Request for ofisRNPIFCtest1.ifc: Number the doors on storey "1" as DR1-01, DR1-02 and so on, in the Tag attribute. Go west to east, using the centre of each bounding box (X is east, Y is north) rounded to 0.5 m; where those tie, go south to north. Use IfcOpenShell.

First a look at what the model holds.

```python
import ifcopenshell
import ifcopenshell.util.element
import ifcopenshell.util.placement

model = ifcopenshell.open("ofisRNPIFCtest1.ifc")
print(model.schema)
storey = next(s for s in model.by_type("IfcBuildingStorey") if s.Name == "1")
doors = [e for e in ifcopenshell.util.element.get_decomposition(storey) if e.is_a("IfcDoor")]
for e in sorted(doors, key=lambda e: e.id()):
    origin = ifcopenshell.util.placement.get_local_placement(e.ObjectPlacement)[:3, 3]
    print(e.id(), e.Tag, e.Name, origin.round(2) + 0.0, sep=" | ")
```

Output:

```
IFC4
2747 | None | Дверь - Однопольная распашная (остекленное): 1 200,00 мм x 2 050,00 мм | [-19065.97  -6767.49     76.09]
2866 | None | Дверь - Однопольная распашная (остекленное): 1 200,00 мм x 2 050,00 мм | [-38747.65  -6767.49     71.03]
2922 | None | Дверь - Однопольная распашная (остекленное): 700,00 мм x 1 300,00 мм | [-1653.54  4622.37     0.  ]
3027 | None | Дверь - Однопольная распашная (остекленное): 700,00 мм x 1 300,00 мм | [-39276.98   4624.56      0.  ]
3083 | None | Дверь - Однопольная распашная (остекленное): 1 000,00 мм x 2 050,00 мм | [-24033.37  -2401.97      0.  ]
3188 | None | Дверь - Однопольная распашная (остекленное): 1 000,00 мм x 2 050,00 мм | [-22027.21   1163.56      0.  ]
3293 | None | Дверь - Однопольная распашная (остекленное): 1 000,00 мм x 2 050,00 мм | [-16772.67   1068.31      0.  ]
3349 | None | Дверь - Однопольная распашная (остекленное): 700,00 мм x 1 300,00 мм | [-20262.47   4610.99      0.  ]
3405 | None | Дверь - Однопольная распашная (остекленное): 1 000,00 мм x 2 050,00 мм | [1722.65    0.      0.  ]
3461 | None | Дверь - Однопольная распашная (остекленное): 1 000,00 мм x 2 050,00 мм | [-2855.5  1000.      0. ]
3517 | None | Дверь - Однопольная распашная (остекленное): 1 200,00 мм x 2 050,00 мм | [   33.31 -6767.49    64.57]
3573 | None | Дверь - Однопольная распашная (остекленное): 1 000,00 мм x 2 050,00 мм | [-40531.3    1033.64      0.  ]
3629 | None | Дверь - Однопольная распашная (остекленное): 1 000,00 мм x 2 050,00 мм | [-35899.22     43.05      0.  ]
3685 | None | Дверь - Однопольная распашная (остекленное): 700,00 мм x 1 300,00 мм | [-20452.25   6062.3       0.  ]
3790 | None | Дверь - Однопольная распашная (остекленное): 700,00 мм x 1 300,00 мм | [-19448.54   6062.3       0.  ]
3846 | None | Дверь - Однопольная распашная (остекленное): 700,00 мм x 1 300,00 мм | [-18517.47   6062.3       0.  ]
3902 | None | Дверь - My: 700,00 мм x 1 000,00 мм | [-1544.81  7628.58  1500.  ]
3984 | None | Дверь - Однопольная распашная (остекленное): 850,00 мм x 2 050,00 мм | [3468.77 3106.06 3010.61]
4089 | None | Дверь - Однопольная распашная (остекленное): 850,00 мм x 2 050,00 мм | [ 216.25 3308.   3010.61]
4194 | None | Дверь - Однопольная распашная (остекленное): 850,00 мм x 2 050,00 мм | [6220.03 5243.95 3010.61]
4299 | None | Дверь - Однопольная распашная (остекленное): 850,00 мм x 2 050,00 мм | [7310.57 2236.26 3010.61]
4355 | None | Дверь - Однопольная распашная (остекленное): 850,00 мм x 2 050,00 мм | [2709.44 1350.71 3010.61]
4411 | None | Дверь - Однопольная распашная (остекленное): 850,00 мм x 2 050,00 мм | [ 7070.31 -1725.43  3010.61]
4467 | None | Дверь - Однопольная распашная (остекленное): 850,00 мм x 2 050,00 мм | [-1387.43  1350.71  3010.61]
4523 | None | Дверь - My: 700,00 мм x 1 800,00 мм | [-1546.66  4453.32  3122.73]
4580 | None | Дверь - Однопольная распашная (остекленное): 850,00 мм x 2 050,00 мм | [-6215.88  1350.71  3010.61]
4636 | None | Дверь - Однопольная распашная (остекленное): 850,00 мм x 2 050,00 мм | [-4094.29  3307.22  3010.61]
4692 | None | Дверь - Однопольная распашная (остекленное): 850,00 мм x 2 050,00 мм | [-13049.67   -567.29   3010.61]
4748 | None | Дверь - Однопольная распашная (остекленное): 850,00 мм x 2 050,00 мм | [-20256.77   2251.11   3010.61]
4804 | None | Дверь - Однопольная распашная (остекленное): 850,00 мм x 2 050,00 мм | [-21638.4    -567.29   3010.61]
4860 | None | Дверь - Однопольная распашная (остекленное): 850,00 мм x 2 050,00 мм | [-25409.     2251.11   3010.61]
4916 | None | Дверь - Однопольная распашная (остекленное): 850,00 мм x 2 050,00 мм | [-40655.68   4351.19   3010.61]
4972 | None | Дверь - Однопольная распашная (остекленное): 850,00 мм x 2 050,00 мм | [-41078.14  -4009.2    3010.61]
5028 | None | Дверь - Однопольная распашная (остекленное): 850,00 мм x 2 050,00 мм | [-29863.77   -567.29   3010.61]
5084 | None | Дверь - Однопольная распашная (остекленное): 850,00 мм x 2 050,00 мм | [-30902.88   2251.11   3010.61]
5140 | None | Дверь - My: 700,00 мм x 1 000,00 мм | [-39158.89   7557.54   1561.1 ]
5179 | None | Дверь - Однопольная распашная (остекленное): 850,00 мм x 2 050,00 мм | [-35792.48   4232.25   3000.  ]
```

```python
import ifcopenshell
import ifcopenshell.geom
import ifcopenshell.util.element
import ifcopenshell.util.shape

model = ifcopenshell.open("ofisRNPIFCtest1.ifc")
settings = ifcopenshell.geom.settings()
settings.set("use-world-coords", True)


def centre(element):
    shape = ifcopenshell.geom.create_shape(settings, element)
    return ifcopenshell.util.shape.get_bbox_centroid(shape.geometry)


storey = next(s for s in model.by_type("IfcBuildingStorey") if s.Name == "1")
doors = [e for e in ifcopenshell.util.element.get_decomposition(storey) if e.is_a("IfcDoor")]

# Insertion points can sit at a corner or the storey origin, so sort by the geometry (in metres).
centres = {e: centre(e) for e in doors}
doors.sort(key=lambda e: (round(centres[e][0] / 0.5), centres[e][1]))

for i, e in enumerate(doors, start=1):
    number = f"DR1-{i:02d}"
    e.Tag = number
    print(e.id(), number)

model.write("ofisRNPIFCtest1_updated.ifc")
```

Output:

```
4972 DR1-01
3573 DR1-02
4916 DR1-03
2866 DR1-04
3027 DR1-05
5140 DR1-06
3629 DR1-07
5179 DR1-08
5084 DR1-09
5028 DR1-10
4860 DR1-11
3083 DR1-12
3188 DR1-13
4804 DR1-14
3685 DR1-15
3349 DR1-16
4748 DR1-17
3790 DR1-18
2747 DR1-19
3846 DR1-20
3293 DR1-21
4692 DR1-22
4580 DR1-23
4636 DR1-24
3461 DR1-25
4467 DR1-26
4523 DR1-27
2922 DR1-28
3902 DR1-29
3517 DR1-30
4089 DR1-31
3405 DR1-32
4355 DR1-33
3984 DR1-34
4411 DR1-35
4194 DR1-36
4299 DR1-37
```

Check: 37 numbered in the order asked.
